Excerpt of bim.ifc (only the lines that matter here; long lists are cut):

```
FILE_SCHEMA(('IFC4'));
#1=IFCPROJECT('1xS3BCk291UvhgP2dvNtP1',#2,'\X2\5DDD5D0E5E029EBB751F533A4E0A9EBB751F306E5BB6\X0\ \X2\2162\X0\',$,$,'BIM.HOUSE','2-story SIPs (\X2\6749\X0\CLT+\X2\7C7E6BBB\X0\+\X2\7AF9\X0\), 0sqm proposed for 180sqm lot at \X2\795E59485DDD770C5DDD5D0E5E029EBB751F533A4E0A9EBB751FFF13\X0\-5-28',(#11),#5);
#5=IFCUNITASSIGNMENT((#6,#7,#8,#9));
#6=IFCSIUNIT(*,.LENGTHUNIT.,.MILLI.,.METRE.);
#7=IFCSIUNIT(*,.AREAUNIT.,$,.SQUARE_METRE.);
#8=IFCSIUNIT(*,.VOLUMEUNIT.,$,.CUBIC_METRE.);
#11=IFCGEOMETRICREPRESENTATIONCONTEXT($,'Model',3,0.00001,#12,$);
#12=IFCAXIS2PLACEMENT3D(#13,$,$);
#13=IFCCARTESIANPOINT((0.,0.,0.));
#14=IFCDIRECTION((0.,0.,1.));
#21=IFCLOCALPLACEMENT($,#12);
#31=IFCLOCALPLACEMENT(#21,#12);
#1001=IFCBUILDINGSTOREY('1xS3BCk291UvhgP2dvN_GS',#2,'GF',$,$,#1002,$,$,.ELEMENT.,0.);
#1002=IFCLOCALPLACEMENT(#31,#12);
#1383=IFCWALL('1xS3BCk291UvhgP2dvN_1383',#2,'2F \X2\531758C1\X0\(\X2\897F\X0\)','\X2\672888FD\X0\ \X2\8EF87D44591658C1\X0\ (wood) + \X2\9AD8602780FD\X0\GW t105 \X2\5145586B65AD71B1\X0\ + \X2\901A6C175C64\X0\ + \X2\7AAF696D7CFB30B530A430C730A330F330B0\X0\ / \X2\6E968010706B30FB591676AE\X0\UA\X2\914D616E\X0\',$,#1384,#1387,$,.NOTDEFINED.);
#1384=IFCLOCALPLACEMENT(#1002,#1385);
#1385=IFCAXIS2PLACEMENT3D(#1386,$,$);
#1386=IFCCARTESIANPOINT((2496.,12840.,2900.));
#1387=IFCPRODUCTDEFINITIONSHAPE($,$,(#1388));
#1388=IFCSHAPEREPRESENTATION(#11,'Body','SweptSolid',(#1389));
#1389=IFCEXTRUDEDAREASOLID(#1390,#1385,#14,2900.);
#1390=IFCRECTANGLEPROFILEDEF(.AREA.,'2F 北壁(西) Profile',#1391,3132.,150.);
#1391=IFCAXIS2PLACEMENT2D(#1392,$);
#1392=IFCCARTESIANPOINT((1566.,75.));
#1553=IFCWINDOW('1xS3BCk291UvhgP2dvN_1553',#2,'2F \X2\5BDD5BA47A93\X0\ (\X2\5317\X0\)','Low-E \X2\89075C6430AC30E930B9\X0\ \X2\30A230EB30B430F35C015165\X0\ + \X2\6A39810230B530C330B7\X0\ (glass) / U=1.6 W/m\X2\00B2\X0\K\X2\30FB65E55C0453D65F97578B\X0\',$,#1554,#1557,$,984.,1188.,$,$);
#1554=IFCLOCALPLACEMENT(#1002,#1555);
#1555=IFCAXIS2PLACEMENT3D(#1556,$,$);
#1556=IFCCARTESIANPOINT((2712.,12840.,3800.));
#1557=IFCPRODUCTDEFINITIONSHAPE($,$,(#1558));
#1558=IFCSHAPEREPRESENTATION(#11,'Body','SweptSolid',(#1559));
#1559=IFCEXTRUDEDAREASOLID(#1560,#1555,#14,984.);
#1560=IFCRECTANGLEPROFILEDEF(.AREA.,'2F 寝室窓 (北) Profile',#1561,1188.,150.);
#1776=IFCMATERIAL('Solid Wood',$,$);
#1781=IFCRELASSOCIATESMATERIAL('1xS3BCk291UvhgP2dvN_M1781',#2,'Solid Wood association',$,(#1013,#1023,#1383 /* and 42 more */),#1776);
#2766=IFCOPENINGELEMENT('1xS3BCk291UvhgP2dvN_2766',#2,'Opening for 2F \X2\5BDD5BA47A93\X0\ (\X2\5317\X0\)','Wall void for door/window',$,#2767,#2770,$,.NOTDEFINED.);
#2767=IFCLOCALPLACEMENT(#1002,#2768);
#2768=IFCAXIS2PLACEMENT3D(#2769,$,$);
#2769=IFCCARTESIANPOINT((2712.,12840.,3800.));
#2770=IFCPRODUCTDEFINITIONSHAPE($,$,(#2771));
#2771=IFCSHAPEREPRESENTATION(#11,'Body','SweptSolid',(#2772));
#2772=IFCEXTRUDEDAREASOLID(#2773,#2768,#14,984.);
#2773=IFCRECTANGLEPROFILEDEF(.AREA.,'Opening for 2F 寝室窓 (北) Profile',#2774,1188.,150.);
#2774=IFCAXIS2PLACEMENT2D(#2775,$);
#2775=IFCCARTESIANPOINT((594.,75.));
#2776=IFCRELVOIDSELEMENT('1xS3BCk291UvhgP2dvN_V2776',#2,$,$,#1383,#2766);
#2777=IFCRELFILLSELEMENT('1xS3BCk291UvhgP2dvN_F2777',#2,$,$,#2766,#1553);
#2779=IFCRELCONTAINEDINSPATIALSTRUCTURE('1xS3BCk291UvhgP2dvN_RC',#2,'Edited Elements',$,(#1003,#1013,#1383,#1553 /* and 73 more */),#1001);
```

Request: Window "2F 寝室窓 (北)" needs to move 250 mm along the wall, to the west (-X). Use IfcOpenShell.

```python
import ifcopenshell
import ifcopenshell.api.geometry
import ifcopenshell.util.placement

model = ifcopenshell.open("bim.ifc")

window = model.by_guid("1xS3BCk291UvhgP2dvN_1553")
opening = window.FillsVoids[0].RelatingOpeningElement
wall = opening.VoidsElements[0].RelatingBuildingElement

wall_matrix = ifcopenshell.util.placement.get_local_placement(wall.ObjectPlacement)
shift = wall_matrix[:3, 0] * -250.0
before = ifcopenshell.util.placement.get_local_placement(window.ObjectPlacement)[:3, 3].copy()

# The window is not placed relative to its opening, so move both.
for product in (opening, window):
    matrix = ifcopenshell.util.placement.get_local_placement(product.ObjectPlacement)
    matrix[:3, 3] += shift
    ifcopenshell.api.geometry.edit_object_placement(model, product=product, matrix=matrix, is_si=False)

after = ifcopenshell.util.placement.get_local_placement(window.ObjectPlacement)[:3, 3]
print("window moved by", (after - before).round(3) + 0.0)

model.write("bim_v2.ifc")
```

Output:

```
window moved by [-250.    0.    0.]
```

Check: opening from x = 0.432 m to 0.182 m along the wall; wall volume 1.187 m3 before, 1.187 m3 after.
